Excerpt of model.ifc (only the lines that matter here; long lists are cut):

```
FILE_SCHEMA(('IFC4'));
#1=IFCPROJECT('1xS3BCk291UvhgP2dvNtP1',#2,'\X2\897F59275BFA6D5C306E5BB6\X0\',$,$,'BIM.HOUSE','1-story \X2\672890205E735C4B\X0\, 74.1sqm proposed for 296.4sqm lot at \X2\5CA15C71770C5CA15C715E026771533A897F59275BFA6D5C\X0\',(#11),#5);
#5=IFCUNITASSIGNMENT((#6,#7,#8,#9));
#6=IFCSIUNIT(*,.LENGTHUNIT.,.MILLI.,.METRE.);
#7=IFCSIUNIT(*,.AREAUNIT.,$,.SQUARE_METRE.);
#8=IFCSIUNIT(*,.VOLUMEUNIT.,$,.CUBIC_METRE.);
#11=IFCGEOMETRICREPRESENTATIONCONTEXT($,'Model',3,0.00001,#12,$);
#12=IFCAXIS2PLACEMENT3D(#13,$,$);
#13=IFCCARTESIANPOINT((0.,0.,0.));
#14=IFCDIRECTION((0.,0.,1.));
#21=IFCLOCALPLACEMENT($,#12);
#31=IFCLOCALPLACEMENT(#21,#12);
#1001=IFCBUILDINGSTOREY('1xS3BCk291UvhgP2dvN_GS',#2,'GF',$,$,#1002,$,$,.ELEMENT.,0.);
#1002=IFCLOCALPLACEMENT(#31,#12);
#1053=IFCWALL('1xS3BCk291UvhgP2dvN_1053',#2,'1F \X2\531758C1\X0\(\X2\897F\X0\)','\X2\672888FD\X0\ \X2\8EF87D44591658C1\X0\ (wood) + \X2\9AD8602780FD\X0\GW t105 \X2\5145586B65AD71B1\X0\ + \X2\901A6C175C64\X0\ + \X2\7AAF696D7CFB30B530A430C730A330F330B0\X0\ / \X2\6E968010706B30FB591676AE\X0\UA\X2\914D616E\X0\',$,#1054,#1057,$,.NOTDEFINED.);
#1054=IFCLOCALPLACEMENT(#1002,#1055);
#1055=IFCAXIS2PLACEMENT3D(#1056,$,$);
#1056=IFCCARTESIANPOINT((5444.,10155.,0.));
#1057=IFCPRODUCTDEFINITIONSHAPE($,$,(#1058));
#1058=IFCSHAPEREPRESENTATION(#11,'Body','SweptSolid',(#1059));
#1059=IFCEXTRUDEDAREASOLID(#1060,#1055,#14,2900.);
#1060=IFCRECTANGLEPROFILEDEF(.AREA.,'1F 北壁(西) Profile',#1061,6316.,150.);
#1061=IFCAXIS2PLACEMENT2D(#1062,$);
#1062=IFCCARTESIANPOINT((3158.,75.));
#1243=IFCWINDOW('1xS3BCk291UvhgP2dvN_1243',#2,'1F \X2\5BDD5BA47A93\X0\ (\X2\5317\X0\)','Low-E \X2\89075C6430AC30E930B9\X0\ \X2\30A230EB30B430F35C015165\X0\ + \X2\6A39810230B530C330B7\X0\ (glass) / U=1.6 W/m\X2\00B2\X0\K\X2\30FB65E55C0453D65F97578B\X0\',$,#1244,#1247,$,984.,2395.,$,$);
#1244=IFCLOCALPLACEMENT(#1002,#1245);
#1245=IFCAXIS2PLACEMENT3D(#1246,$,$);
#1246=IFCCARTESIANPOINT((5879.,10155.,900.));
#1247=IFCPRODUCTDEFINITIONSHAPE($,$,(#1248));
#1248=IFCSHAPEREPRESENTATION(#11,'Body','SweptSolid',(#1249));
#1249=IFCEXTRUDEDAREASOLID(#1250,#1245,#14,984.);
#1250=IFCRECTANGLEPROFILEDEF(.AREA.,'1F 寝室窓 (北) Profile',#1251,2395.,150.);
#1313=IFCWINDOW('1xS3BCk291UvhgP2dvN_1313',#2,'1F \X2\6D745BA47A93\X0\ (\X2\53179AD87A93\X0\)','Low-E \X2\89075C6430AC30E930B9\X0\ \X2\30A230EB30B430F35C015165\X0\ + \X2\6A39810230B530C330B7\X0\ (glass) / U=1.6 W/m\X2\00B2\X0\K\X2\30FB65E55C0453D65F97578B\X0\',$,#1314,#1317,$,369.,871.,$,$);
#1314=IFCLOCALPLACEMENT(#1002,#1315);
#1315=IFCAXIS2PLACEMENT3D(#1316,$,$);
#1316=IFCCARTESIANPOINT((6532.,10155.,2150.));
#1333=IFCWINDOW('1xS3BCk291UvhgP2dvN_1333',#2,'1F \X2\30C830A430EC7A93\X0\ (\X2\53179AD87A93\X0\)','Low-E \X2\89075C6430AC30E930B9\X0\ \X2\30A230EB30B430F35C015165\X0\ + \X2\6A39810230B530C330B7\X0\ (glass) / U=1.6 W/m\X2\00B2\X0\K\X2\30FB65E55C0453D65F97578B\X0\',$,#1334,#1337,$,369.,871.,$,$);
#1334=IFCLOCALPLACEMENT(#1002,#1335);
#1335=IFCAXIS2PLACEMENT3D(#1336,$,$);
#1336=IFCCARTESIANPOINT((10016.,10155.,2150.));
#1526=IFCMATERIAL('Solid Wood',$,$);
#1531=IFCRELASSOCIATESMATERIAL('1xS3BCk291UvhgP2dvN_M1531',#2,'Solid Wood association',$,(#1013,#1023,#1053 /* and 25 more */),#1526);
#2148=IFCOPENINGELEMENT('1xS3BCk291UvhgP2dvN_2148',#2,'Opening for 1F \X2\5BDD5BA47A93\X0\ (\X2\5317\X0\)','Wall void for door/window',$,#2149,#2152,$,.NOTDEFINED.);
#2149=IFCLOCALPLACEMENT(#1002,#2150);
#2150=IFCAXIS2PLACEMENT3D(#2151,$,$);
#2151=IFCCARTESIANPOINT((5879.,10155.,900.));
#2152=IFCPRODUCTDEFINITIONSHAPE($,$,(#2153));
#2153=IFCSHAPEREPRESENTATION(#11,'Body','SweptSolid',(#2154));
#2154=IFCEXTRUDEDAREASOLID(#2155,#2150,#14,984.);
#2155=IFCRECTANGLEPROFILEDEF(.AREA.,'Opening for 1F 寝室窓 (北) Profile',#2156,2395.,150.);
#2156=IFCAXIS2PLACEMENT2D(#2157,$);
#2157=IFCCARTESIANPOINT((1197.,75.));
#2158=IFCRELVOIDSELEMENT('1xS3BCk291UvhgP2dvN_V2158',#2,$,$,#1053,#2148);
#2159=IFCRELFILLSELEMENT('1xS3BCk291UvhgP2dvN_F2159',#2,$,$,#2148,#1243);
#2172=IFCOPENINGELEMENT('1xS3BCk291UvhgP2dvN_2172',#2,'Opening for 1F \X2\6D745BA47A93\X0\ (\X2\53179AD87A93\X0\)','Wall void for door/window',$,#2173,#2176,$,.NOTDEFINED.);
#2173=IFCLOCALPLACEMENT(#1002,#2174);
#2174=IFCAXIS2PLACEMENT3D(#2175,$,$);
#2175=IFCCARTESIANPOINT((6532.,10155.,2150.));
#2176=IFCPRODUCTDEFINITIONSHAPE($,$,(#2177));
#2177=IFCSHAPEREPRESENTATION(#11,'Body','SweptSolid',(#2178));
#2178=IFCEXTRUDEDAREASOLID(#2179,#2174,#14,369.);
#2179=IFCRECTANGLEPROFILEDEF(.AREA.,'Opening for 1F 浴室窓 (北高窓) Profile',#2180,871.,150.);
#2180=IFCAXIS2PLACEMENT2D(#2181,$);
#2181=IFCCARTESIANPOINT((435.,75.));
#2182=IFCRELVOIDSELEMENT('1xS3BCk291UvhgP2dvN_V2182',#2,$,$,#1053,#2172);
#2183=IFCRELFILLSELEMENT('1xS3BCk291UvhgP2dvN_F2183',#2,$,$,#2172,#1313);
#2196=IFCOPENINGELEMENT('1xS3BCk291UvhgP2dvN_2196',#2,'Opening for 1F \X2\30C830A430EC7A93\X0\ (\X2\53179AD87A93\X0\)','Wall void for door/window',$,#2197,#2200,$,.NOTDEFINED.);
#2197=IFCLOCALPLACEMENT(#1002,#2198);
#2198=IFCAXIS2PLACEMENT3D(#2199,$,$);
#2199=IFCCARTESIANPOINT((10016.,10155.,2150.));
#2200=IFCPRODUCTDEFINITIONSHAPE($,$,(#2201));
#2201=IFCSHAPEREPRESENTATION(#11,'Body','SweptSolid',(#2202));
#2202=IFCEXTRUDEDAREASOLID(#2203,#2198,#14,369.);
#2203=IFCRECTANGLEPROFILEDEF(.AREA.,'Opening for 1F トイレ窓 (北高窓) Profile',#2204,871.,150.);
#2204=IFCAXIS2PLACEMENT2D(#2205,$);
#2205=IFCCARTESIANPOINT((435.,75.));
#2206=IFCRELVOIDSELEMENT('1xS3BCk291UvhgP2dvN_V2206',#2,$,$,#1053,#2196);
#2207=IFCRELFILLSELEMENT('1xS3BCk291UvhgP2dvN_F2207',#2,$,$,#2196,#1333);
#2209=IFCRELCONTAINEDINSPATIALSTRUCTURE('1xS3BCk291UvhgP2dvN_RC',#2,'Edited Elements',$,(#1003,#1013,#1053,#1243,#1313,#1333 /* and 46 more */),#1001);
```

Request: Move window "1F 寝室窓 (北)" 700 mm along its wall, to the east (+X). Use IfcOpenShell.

```python
import ifcopenshell
import ifcopenshell.api.geometry
import ifcopenshell.util.placement
import ifcopenshell.util.unit

model = ifcopenshell.open("model.ifc")
unit_scale = ifcopenshell.util.unit.calculate_unit_scale(model)

window = model.by_id(1243)
opening = window.FillsVoids[0].RelatingOpeningElement
wall = opening.VoidsElements[0].RelatingBuildingElement

wall_matrix = ifcopenshell.util.placement.get_local_placement(wall.ObjectPlacement)
shift = wall_matrix[:3, 0] * 0.7 / unit_scale
before = ifcopenshell.util.placement.get_local_placement(window.ObjectPlacement)[:3, 3].copy()

# The window is not placed relative to its opening, so move both.
for product in (opening, window):
    matrix = ifcopenshell.util.placement.get_local_placement(product.ObjectPlacement)
    matrix[:3, 3] += shift
    ifcopenshell.api.geometry.edit_object_placement(model, product=product, matrix=matrix, is_si=False)

after = ifcopenshell.util.placement.get_local_placement(window.ObjectPlacement)[:3, 3]
print("window moved by", (after - before).round(3) + 0.0)

model.write("model_updated.ifc")
```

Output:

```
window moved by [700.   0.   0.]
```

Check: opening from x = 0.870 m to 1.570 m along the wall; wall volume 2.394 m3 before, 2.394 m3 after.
